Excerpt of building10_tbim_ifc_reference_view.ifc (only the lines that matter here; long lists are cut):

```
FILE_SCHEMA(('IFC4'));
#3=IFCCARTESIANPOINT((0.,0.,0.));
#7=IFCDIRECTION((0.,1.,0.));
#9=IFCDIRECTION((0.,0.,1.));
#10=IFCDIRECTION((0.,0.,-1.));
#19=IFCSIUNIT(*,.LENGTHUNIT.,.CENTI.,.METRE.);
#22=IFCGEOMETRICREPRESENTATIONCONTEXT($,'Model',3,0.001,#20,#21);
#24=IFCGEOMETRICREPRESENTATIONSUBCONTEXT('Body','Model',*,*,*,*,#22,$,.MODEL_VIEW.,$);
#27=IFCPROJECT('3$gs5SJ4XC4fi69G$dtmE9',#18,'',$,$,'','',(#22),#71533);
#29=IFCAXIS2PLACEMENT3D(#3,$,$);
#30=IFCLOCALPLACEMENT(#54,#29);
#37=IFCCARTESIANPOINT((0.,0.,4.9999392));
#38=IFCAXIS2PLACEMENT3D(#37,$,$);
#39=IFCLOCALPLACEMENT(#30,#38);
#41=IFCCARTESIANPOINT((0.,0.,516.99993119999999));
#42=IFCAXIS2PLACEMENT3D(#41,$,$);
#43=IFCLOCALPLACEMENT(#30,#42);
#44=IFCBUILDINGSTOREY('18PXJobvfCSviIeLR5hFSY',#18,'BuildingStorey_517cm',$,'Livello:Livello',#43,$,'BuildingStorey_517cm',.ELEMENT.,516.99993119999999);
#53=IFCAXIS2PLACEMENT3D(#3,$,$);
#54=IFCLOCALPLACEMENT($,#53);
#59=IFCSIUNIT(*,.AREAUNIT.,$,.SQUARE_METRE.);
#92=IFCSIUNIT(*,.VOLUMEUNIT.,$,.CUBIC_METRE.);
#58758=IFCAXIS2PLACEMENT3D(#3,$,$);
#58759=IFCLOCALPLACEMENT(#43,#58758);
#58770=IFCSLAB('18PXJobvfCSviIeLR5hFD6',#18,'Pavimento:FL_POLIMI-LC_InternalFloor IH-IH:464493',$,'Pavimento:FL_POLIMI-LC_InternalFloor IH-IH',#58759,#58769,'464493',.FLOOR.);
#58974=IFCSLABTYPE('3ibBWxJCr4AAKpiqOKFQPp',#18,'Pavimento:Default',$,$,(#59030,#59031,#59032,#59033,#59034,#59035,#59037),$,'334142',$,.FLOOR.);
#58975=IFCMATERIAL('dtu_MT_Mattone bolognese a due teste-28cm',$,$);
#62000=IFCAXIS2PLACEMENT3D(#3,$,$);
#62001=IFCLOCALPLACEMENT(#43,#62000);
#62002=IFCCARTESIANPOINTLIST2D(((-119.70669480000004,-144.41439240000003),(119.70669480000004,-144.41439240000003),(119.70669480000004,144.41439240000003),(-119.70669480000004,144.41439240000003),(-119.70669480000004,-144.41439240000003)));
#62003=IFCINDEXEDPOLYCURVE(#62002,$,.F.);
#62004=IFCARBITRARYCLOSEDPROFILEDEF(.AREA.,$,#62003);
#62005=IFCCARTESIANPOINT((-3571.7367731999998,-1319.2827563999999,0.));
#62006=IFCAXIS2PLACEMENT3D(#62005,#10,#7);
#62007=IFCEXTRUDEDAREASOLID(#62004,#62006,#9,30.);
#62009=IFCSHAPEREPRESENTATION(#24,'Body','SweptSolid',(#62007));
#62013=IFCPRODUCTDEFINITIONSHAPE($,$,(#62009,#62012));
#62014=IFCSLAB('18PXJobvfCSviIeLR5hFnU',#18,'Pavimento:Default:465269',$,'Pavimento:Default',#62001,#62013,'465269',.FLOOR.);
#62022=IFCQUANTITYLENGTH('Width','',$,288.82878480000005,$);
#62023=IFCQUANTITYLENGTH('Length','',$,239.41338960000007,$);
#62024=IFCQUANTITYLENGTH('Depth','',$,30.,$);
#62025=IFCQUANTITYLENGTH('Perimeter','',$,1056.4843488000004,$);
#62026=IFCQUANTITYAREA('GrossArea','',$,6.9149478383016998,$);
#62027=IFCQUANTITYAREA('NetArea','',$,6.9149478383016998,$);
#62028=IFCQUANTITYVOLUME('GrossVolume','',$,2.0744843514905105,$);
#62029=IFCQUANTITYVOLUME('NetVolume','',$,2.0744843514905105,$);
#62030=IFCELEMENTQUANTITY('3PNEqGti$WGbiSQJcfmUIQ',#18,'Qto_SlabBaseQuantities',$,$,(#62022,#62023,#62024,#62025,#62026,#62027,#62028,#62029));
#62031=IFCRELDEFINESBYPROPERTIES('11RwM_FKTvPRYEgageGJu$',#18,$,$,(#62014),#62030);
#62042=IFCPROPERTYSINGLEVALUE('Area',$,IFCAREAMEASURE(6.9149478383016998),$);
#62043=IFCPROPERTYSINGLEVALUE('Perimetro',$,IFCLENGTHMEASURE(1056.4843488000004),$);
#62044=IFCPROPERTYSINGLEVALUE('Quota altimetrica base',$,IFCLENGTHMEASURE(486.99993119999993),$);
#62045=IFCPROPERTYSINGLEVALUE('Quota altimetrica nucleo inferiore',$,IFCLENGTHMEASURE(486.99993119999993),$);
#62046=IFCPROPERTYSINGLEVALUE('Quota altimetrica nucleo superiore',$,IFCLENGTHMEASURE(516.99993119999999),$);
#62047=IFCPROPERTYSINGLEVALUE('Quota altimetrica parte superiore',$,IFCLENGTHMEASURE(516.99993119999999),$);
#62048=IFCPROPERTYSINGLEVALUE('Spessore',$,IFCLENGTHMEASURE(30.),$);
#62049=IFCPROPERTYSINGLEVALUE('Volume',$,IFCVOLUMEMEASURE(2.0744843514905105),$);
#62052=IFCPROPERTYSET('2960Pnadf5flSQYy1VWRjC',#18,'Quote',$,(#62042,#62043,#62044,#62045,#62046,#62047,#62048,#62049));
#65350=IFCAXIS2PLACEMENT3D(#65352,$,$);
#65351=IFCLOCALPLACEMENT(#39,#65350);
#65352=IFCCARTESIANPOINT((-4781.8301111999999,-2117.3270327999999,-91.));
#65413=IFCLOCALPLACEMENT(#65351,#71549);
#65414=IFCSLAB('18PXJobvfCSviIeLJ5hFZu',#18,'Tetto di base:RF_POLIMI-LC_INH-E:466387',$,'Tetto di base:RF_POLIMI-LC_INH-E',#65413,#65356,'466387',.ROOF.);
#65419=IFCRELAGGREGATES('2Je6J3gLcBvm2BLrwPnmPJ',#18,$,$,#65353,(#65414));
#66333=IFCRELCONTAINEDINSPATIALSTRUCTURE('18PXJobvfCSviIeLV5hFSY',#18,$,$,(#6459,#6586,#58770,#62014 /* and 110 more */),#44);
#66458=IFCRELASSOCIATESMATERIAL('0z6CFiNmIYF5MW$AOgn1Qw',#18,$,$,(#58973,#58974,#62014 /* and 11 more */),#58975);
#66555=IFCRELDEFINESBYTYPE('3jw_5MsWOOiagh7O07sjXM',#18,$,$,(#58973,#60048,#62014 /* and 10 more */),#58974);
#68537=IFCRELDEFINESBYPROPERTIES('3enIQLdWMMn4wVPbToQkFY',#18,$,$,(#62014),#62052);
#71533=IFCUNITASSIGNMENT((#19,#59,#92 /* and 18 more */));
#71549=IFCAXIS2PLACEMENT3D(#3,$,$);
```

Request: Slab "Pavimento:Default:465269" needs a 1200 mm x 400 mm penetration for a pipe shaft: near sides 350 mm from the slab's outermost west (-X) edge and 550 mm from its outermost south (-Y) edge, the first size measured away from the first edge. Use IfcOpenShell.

```python
import numpy as np
import ifcopenshell
import ifcopenshell.api.feature
import ifcopenshell.api.geometry
import ifcopenshell.api.pset
import ifcopenshell.api.root
import ifcopenshell.geom
import ifcopenshell.util.element
import ifcopenshell.util.placement
import ifcopenshell.util.representation
import ifcopenshell.util.shape
import ifcopenshell.util.unit

model = ifcopenshell.open("building10_tbim_ifc_reference_view.ifc")
unit_scale = ifcopenshell.util.unit.calculate_unit_scale(model)
area_scale = ifcopenshell.util.unit.calculate_unit_scale(model, "AREAUNIT")
volume_scale = ifcopenshell.util.unit.calculate_unit_scale(model, "VOLUMEUNIT")
settings = ifcopenshell.geom.settings()


def volume(element):
    """Net volume in cubic metres, openings subtracted."""
    shape = ifcopenshell.geom.create_shape(settings, element)
    return ifcopenshell.util.shape.get_volume(shape.geometry)


slab = model.by_guid("18PXJobvfCSviIeLR5hFnU")
before = volume(slab)

# Extent in the slab's own axes, in metres. The edges named are its -X and -Y sides.
slab_shape = ifcopenshell.geom.create_shape(settings, slab)
vertices = ifcopenshell.util.shape.get_vertices(slab_shape.geometry)
x_min, y_min, bottom = vertices.min(axis=0)
top = vertices[:, 2].max()

opening = ifcopenshell.api.root.create_entity(model, ifc_class="IfcOpeningElement", name="Pipe shaft opening", predefined_type="OPENING")
context = ifcopenshell.util.representation.get_context(model, "Model", "Body", "MODEL_VIEW")
width, depth = 1.2, 0.4
outline = [(0.0, 0.0), (width, 0.0), (width, depth), (0.0, depth), (0.0, 0.0)]
# Overshoot both faces by 50 mm so the cut is clean.
shape = ifcopenshell.api.geometry.add_slab_representation(
    model, context=context, depth=top - bottom + 0.1, polyline=outline
)
ifcopenshell.api.geometry.assign_representation(model, product=opening, representation=shape)

matrix = ifcopenshell.util.placement.get_local_placement(slab.ObjectPlacement)
matrix[:, 3] = matrix @ np.append(np.array([x_min + 0.35, y_min + 0.55, bottom - 0.05]) / unit_scale, 1.0)
ifcopenshell.api.geometry.edit_object_placement(model, product=opening, matrix=matrix, is_si=False)
ifcopenshell.api.feature.add_feature(model, feature=opening, element=slab)

after = volume(slab)

# Update the slab's stored quantities.
qto = model.by_id(ifcopenshell.util.element.get_pset(slab, "Qto_SlabBaseQuantities", should_inherit=False)["id"])
ifcopenshell.api.pset.edit_qto(model, qto=qto, properties={
    "NetArea": after / (top - bottom) / area_scale,
    "NetVolume": after / volume_scale,
})
pset = model.by_id(ifcopenshell.util.element.get_pset(slab, "Quote", should_inherit=False)["id"])
ifcopenshell.api.pset.edit_pset(model, pset=pset, properties={
    "Area": model.create_entity("IfcAreaMeasure", after / (top - bottom) / area_scale),
    "Volume": model.create_entity("IfcVolumeMeasure", after / volume_scale),
})

print(f"slab volume {before:.3f} -> {after:.3f} m3")

model.write("building10_tbim_ifc_reference_view-out.ifc")
```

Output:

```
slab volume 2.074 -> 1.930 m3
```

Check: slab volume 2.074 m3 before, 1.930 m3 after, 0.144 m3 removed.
